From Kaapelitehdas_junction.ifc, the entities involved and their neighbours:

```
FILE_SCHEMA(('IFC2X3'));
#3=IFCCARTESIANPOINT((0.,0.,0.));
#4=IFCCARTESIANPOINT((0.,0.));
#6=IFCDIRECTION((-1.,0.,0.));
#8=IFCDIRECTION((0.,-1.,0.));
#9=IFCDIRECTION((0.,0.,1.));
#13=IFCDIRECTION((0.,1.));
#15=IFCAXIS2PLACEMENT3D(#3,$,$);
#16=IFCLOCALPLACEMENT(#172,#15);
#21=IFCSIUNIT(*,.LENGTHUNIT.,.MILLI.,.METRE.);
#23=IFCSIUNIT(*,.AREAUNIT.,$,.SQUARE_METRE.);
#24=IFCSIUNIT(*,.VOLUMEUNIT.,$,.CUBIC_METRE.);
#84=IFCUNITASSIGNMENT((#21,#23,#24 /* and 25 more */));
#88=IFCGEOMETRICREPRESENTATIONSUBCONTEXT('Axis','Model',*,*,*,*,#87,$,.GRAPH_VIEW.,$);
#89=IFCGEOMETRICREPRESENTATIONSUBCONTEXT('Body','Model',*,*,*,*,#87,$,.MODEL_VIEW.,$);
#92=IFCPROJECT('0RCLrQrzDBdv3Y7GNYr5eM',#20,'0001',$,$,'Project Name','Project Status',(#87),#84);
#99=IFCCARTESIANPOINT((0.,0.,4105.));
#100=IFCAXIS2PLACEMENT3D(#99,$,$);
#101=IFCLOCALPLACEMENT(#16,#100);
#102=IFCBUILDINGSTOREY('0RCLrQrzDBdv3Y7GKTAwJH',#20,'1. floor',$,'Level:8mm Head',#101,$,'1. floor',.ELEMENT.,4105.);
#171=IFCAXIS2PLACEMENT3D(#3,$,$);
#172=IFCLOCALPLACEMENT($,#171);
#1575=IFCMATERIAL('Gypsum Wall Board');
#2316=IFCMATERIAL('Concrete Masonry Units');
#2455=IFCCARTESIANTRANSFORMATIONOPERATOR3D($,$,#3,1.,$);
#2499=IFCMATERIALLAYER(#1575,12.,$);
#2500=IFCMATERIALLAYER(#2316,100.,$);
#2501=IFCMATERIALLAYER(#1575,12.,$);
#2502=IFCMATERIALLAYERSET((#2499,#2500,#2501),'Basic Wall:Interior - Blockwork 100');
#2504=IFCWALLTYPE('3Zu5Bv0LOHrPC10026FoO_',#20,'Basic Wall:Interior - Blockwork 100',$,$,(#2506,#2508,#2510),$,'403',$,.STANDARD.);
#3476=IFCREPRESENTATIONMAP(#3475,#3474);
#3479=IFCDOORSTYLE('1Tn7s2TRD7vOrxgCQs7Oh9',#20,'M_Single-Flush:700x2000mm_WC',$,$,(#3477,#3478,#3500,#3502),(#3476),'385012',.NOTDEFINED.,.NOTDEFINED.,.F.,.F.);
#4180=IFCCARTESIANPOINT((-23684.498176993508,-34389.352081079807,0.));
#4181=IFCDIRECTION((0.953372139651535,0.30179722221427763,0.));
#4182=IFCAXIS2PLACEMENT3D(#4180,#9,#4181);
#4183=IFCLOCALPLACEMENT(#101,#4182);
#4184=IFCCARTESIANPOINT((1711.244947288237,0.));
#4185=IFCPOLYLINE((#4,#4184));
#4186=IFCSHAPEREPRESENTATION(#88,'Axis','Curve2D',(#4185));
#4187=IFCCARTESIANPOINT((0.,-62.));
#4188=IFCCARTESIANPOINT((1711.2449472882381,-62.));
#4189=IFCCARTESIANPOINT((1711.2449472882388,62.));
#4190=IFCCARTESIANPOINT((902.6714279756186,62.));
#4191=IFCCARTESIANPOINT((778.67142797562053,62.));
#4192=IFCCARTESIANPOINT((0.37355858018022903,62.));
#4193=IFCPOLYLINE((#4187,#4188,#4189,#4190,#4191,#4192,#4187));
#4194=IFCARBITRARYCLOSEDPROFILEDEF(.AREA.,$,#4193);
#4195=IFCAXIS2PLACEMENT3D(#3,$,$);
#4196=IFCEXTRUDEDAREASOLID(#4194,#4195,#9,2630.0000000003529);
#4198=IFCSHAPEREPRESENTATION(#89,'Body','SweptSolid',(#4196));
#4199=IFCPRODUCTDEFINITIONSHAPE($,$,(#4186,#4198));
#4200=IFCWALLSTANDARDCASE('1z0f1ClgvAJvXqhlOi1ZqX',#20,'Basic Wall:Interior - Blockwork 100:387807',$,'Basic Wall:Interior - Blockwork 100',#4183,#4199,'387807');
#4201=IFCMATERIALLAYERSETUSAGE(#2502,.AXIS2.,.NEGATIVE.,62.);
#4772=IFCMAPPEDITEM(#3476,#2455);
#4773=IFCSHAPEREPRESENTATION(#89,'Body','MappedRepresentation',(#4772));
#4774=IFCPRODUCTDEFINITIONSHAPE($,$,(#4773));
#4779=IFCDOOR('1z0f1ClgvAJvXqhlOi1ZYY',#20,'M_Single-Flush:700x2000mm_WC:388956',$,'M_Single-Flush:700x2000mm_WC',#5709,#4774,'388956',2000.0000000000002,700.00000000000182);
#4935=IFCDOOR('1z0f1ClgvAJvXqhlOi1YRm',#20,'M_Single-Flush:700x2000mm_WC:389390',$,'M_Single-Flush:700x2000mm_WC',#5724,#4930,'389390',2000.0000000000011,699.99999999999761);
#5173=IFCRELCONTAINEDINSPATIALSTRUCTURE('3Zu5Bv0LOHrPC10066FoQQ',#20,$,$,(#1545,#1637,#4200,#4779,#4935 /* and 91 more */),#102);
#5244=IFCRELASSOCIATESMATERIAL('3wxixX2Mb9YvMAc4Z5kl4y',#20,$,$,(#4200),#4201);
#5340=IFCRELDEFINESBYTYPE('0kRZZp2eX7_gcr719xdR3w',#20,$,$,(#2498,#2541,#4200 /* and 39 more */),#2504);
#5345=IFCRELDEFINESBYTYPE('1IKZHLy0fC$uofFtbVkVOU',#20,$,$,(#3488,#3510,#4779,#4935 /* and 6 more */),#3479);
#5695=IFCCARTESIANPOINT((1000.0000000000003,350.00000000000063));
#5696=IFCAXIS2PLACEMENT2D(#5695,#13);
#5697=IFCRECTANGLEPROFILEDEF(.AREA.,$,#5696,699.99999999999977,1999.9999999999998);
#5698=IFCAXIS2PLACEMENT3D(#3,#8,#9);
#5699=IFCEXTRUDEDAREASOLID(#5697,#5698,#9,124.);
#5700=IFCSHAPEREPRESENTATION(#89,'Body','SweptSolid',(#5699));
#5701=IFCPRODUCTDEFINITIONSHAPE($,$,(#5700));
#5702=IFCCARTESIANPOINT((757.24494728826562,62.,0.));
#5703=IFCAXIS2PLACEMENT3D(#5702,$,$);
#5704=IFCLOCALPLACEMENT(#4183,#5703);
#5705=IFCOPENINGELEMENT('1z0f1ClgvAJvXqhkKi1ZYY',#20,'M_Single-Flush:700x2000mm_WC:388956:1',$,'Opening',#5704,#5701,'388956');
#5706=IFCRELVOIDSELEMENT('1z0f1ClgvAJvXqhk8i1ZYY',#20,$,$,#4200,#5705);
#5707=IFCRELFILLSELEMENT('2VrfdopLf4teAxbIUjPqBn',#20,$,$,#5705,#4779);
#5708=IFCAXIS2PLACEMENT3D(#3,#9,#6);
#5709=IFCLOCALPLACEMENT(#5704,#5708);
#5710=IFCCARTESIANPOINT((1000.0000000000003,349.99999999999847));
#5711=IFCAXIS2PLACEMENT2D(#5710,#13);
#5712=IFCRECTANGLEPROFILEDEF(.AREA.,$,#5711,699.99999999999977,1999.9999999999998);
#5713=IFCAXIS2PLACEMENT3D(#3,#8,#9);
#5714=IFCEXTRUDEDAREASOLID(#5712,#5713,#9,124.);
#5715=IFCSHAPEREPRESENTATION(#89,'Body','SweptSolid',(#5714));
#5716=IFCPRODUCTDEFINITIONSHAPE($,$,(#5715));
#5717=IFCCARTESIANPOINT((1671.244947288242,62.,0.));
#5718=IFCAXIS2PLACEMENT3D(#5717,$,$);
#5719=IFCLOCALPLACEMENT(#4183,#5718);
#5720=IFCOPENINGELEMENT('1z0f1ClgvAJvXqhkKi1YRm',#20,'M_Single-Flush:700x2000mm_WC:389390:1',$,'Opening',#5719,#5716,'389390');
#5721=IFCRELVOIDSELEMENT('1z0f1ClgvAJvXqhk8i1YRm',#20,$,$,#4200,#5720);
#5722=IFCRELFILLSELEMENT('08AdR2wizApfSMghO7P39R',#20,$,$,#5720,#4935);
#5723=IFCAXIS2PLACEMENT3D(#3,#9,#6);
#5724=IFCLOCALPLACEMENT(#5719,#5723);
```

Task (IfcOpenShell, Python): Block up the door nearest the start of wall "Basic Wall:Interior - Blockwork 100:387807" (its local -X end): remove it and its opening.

```python
import ifcopenshell
import ifcopenshell.api.feature
import ifcopenshell.api.root
import ifcopenshell.geom
import ifcopenshell.util.shape

model = ifcopenshell.open("Kaapelitehdas_junction.ifc")
settings = ifcopenshell.geom.settings()


def volume(element):
    """Net volume in cubic metres, openings subtracted."""
    shape = ifcopenshell.geom.create_shape(settings, element)
    return ifcopenshell.util.shape.get_volume(shape.geometry)


door = model.by_id(4779)
opening = door.FillsVoids[0].RelatingOpeningElement
wall = opening.VoidsElements[0].RelatingBuildingElement
before = volume(wall)

ifcopenshell.api.root.remove_product(model, product=door)
ifcopenshell.api.feature.remove_feature(model, feature=opening)

after = volume(wall)

print(f"wall volume {before:.3f} -> {after:.3f} m3")

model.write("Kaapelitehdas_junction_edited.ifc")
```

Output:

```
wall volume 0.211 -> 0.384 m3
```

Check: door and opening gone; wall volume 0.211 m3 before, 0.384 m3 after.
